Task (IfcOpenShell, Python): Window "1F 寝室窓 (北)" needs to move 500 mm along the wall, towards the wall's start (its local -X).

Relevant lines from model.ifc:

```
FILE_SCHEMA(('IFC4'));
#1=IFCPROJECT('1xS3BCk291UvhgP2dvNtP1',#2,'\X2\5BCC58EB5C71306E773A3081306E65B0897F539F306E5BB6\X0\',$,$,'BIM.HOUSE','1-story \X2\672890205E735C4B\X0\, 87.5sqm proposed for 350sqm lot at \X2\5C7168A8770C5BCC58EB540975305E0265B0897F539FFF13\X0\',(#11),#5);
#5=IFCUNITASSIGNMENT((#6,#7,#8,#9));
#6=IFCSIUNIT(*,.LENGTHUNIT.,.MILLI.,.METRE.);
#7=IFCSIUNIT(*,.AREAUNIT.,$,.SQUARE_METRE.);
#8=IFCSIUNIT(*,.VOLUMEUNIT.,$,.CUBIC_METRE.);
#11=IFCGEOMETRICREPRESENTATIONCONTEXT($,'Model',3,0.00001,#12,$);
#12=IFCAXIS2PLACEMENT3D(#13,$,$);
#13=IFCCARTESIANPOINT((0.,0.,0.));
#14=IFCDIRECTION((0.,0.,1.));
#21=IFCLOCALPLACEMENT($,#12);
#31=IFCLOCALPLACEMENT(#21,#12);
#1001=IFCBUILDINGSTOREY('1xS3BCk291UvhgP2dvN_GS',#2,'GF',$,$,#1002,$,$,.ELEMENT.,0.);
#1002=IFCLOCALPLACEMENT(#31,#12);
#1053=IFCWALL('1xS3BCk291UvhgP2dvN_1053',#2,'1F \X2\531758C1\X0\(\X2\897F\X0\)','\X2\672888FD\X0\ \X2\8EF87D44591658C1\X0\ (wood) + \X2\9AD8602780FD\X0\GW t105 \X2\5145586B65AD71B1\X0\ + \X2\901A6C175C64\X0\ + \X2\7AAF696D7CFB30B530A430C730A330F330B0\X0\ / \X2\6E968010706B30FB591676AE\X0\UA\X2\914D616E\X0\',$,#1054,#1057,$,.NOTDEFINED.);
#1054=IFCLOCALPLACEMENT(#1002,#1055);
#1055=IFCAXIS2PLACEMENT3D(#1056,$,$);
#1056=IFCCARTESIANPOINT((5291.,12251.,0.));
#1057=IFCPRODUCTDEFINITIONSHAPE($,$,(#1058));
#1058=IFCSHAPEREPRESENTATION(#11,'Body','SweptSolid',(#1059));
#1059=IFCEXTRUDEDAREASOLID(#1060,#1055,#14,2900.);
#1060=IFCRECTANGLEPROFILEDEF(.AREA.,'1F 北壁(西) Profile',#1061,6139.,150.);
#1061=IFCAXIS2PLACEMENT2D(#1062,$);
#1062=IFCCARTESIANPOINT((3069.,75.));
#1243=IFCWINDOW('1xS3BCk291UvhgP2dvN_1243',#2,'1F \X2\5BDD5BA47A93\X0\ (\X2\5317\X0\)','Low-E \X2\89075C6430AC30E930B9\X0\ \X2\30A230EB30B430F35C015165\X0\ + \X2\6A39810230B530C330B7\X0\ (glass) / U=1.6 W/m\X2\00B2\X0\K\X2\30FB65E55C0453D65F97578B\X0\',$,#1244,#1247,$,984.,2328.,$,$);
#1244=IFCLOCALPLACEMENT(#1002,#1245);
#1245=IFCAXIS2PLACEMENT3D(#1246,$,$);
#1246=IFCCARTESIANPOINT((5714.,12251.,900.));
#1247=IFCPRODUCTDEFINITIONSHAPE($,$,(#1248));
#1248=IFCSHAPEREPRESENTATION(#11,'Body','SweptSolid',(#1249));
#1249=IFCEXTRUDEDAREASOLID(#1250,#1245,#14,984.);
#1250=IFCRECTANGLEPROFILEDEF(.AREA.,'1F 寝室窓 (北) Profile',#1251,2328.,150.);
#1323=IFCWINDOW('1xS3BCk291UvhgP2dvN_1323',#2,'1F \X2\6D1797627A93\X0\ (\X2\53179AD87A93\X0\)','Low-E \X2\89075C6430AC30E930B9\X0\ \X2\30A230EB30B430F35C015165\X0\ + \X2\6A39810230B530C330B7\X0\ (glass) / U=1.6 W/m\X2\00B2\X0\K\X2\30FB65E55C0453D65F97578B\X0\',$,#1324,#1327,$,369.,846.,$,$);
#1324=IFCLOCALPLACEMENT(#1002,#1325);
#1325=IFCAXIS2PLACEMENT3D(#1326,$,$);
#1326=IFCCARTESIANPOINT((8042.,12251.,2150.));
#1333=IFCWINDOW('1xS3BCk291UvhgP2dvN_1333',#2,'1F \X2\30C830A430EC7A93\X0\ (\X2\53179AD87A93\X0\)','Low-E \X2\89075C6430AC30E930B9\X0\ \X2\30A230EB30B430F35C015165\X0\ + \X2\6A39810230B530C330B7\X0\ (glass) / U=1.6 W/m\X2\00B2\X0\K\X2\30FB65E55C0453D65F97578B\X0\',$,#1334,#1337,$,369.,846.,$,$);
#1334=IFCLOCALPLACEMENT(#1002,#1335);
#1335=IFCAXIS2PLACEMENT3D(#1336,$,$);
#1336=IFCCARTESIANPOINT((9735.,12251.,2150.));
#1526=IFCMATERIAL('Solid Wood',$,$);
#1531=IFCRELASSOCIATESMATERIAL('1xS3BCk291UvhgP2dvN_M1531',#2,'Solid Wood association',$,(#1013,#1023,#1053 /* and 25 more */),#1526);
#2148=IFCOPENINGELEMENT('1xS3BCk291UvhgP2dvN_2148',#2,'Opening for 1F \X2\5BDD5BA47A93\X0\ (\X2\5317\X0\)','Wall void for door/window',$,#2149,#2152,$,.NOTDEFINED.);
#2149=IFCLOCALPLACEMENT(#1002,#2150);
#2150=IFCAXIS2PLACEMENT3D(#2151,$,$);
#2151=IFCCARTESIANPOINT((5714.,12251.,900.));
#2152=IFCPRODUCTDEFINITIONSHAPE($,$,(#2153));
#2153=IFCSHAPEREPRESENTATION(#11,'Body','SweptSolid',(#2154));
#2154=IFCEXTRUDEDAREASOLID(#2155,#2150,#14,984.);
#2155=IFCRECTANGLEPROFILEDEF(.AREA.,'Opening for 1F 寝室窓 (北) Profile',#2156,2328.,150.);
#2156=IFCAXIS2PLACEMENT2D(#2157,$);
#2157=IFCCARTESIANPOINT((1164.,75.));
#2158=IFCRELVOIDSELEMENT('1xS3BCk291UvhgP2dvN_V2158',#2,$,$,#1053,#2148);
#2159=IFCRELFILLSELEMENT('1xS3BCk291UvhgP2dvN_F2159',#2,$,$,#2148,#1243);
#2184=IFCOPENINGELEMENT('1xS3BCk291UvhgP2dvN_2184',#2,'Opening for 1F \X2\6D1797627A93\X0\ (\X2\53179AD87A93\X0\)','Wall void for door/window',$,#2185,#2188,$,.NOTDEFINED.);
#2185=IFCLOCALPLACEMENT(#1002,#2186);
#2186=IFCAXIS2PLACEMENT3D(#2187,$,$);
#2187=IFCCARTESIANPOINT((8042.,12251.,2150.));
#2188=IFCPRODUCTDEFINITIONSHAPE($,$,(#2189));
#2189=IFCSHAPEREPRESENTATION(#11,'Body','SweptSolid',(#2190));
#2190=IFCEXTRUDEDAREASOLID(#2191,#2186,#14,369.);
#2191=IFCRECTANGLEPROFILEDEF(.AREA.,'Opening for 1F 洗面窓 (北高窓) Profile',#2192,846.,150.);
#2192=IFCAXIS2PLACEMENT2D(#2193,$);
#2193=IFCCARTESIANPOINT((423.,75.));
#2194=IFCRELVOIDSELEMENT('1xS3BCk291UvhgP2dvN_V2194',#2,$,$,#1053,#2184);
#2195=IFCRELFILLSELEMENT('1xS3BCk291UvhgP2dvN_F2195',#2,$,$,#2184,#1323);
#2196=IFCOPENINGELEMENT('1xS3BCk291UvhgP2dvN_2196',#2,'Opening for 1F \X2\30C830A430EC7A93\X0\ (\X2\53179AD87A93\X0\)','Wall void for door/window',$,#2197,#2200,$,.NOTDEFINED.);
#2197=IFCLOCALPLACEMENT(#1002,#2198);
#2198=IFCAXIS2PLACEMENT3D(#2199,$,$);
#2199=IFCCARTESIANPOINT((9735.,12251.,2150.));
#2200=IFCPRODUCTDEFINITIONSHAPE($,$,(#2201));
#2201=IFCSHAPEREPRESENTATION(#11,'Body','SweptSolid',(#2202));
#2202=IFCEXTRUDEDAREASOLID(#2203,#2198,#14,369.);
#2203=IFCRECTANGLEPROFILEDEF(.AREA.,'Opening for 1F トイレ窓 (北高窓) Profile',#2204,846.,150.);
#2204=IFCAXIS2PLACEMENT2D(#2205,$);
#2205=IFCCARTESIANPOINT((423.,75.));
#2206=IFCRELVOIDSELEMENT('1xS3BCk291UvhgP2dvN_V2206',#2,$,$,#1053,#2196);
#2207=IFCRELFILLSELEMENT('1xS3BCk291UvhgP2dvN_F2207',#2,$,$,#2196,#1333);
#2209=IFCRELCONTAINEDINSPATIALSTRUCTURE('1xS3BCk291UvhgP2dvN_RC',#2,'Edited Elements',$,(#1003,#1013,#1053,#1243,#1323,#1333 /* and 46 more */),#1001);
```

```python
import ifcopenshell
import ifcopenshell.api.geometry
import ifcopenshell.util.placement
import ifcopenshell.util.unit

model = ifcopenshell.open("model.ifc")
unit_scale = ifcopenshell.util.unit.calculate_unit_scale(model)

window = model.by_id(1243)
opening = window.FillsVoids[0].RelatingOpeningElement
wall = opening.VoidsElements[0].RelatingBuildingElement

wall_matrix = ifcopenshell.util.placement.get_local_placement(wall.ObjectPlacement)
shift = wall_matrix[:3, 0] * -0.5 / unit_scale
before = ifcopenshell.util.placement.get_local_placement(window.ObjectPlacement)[:3, 3].copy()

# The window is not placed relative to its opening, so move both.
for product in (opening, window):
    matrix = ifcopenshell.util.placement.get_local_placement(product.ObjectPlacement)
    matrix[:3, 3] += shift
    ifcopenshell.api.geometry.edit_object_placement(model, product=product, matrix=matrix, is_si=False)

after = ifcopenshell.util.placement.get_local_placement(window.ObjectPlacement)[:3, 3]
print("window moved by", (after - before).round(3) + 0.0)

model.write("model_v2.ifc")
```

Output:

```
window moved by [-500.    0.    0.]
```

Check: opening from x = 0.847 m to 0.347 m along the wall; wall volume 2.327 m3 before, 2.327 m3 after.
